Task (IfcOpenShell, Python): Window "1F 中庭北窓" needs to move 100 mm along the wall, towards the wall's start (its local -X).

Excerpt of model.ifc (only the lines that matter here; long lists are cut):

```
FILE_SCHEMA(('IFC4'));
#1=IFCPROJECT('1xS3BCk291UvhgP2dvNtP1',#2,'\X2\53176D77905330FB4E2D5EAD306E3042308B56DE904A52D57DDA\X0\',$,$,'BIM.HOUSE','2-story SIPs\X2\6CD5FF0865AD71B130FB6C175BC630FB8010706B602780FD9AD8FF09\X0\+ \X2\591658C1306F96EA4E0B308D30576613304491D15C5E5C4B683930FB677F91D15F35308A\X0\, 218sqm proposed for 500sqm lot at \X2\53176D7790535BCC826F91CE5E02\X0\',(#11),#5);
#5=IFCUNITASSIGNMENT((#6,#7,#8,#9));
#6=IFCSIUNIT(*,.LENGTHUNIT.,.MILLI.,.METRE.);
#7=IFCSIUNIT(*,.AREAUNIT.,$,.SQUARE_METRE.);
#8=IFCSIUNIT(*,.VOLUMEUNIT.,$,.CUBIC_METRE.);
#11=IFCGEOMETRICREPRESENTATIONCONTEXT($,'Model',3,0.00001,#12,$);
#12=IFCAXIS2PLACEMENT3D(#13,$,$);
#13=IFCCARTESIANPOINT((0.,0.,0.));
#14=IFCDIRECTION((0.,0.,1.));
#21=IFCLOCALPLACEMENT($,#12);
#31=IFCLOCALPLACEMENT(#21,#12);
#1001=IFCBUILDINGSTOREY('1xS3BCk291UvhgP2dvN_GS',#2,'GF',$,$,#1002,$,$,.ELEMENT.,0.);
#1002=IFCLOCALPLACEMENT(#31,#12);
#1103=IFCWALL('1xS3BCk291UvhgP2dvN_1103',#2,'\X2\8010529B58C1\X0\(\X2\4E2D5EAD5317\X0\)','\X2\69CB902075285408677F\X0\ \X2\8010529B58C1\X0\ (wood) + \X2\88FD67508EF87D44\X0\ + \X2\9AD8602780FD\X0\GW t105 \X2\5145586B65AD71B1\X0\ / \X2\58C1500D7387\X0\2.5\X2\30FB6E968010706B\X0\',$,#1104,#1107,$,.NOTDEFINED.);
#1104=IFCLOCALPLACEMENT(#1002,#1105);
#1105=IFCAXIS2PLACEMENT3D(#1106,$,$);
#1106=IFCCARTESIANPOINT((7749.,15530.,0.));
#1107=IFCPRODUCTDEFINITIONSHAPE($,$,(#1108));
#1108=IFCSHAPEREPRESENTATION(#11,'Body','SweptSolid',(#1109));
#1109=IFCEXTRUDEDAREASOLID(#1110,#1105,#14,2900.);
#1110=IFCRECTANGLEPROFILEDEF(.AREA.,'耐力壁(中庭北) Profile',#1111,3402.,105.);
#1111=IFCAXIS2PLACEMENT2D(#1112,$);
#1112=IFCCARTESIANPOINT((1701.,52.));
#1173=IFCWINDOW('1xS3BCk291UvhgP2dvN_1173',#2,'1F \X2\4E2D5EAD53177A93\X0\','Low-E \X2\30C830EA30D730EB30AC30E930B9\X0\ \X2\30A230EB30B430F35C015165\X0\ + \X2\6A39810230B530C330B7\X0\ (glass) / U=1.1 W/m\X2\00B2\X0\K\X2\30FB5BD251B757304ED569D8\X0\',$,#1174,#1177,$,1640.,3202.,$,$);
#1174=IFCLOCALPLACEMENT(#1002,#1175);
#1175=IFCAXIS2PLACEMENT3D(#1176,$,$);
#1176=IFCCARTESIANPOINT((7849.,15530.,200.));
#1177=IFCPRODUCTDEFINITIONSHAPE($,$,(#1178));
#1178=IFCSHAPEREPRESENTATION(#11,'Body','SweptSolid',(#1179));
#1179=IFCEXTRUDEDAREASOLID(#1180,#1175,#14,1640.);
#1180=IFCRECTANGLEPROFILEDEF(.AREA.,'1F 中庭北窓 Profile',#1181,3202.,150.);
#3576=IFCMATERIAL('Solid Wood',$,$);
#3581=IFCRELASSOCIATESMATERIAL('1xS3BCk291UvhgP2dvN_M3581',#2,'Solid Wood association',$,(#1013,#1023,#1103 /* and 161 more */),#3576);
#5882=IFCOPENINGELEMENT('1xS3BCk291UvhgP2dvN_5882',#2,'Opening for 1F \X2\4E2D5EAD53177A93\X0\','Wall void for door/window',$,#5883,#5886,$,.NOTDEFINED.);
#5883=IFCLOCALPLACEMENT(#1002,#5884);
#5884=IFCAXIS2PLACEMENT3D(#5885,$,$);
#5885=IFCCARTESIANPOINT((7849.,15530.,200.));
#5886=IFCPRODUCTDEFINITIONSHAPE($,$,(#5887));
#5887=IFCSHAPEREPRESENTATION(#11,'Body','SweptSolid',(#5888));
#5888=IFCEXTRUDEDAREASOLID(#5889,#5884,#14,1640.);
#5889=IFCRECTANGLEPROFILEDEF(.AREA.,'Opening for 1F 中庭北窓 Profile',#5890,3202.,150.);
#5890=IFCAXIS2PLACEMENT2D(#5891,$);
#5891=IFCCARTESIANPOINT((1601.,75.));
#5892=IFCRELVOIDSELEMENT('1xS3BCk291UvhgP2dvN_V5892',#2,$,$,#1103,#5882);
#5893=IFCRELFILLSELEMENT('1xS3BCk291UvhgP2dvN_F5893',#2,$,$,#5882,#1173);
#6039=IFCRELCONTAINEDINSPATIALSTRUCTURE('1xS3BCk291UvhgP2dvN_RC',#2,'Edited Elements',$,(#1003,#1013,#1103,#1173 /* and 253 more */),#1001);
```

```python
import ifcopenshell
import ifcopenshell.api.geometry
import ifcopenshell.util.placement
import ifcopenshell.util.unit

model = ifcopenshell.open("model.ifc")
unit_scale = ifcopenshell.util.unit.calculate_unit_scale(model)

window = model.by_guid("1xS3BCk291UvhgP2dvN_1173")
opening = window.FillsVoids[0].RelatingOpeningElement
wall = opening.VoidsElements[0].RelatingBuildingElement

wall_matrix = ifcopenshell.util.placement.get_local_placement(wall.ObjectPlacement)
shift = wall_matrix[:3, 0] * -0.1 / unit_scale
before = ifcopenshell.util.placement.get_local_placement(window.ObjectPlacement)[:3, 3].copy()

# The window is not placed relative to its opening, so move both.
for product in (opening, window):
    matrix = ifcopenshell.util.placement.get_local_placement(product.ObjectPlacement)
    matrix[:3, 3] += shift
    ifcopenshell.api.geometry.edit_object_placement(model, product=product, matrix=matrix, is_si=False)

after = ifcopenshell.util.placement.get_local_placement(window.ObjectPlacement)[:3, 3]
print("window moved by", (after - before).round(3) + 0.0)

model.write("model_updated.ifc")
```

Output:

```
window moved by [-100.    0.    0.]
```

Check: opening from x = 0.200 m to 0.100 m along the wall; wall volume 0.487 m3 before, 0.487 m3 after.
